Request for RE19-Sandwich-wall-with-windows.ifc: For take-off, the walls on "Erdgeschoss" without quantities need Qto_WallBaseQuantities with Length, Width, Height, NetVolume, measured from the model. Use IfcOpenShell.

First a look at what the model holds.

```python
import ifcopenshell
import ifcopenshell.util.element
import ifcopenshell.util.unit

model = ifcopenshell.open("RE19-Sandwich-wall-with-windows.ifc")
print(model.schema)
for unit_type in ("LENGTHUNIT", "AREAUNIT", "VOLUMEUNIT"):
    print(unit_type, ifcopenshell.util.unit.calculate_unit_scale(model, unit_type))
storey = next(s for s in model.by_type("IfcBuildingStorey") if s.Name == "Erdgeschoss")
walls = [e for e in ifcopenshell.util.element.get_decomposition(storey) if e.is_a("IfcWall")]
for e in sorted(walls, key=lambda e: e.id()):
    print(e.id(), e.is_a(), e.Name, list(ifcopenshell.util.element.get_psets(e, qtos_only=True)), sep=" | ")
```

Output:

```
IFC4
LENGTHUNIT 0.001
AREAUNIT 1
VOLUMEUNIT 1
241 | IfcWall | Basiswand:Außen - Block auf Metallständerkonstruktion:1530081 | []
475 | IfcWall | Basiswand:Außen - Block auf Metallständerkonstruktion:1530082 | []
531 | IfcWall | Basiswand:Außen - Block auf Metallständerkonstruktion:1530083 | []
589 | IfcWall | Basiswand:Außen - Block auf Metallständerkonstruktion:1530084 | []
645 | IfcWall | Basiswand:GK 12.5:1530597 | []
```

```python
import ifcopenshell
import ifcopenshell.api.pset
import ifcopenshell.geom
import ifcopenshell.util.element
import ifcopenshell.util.shape
import ifcopenshell.util.unit

model = ifcopenshell.open("RE19-Sandwich-wall-with-windows.ifc")
unit_scale = ifcopenshell.util.unit.calculate_unit_scale(model)
volume_scale = ifcopenshell.util.unit.calculate_unit_scale(model, "VOLUMEUNIT")
settings = ifcopenshell.geom.settings()

storey = next(s for s in model.by_type("IfcBuildingStorey") if s.Name == "Erdgeschoss")
walls = [e for e in ifcopenshell.util.element.get_decomposition(storey) if e.is_a("IfcWall")]

for e in sorted(walls, key=lambda e: e.id()):
    if ifcopenshell.util.element.get_psets(e, qtos_only=True, should_inherit=False):
        continue
    # Geometry comes back in metres, in the element's own axes.
    shape = ifcopenshell.geom.create_shape(settings, e)
    values = {
        "Length": ifcopenshell.util.shape.get_x(shape.geometry) / unit_scale,
        "Width": ifcopenshell.util.shape.get_y(shape.geometry) / unit_scale,
        "Height": ifcopenshell.util.shape.get_z(shape.geometry) / unit_scale,
        "NetVolume": ifcopenshell.util.shape.get_volume(shape.geometry) / volume_scale,
    }
    qto = ifcopenshell.api.pset.add_qto(model, product=e, name="Qto_WallBaseQuantities")
    ifcopenshell.api.pset.edit_qto(model, qto=qto, properties=values)
    print(e.id(), {k: round(v, 3) for k, v in values.items()})

model.write("RE19-Sandwich-wall-with-windows_edited.ifc")
```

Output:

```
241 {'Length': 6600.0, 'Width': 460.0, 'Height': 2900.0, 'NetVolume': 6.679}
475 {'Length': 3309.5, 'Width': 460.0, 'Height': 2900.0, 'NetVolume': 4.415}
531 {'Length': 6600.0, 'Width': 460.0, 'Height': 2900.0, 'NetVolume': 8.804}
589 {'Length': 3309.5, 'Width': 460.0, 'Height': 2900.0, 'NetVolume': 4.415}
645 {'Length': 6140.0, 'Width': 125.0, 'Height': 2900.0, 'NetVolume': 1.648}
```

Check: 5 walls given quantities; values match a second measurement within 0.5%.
